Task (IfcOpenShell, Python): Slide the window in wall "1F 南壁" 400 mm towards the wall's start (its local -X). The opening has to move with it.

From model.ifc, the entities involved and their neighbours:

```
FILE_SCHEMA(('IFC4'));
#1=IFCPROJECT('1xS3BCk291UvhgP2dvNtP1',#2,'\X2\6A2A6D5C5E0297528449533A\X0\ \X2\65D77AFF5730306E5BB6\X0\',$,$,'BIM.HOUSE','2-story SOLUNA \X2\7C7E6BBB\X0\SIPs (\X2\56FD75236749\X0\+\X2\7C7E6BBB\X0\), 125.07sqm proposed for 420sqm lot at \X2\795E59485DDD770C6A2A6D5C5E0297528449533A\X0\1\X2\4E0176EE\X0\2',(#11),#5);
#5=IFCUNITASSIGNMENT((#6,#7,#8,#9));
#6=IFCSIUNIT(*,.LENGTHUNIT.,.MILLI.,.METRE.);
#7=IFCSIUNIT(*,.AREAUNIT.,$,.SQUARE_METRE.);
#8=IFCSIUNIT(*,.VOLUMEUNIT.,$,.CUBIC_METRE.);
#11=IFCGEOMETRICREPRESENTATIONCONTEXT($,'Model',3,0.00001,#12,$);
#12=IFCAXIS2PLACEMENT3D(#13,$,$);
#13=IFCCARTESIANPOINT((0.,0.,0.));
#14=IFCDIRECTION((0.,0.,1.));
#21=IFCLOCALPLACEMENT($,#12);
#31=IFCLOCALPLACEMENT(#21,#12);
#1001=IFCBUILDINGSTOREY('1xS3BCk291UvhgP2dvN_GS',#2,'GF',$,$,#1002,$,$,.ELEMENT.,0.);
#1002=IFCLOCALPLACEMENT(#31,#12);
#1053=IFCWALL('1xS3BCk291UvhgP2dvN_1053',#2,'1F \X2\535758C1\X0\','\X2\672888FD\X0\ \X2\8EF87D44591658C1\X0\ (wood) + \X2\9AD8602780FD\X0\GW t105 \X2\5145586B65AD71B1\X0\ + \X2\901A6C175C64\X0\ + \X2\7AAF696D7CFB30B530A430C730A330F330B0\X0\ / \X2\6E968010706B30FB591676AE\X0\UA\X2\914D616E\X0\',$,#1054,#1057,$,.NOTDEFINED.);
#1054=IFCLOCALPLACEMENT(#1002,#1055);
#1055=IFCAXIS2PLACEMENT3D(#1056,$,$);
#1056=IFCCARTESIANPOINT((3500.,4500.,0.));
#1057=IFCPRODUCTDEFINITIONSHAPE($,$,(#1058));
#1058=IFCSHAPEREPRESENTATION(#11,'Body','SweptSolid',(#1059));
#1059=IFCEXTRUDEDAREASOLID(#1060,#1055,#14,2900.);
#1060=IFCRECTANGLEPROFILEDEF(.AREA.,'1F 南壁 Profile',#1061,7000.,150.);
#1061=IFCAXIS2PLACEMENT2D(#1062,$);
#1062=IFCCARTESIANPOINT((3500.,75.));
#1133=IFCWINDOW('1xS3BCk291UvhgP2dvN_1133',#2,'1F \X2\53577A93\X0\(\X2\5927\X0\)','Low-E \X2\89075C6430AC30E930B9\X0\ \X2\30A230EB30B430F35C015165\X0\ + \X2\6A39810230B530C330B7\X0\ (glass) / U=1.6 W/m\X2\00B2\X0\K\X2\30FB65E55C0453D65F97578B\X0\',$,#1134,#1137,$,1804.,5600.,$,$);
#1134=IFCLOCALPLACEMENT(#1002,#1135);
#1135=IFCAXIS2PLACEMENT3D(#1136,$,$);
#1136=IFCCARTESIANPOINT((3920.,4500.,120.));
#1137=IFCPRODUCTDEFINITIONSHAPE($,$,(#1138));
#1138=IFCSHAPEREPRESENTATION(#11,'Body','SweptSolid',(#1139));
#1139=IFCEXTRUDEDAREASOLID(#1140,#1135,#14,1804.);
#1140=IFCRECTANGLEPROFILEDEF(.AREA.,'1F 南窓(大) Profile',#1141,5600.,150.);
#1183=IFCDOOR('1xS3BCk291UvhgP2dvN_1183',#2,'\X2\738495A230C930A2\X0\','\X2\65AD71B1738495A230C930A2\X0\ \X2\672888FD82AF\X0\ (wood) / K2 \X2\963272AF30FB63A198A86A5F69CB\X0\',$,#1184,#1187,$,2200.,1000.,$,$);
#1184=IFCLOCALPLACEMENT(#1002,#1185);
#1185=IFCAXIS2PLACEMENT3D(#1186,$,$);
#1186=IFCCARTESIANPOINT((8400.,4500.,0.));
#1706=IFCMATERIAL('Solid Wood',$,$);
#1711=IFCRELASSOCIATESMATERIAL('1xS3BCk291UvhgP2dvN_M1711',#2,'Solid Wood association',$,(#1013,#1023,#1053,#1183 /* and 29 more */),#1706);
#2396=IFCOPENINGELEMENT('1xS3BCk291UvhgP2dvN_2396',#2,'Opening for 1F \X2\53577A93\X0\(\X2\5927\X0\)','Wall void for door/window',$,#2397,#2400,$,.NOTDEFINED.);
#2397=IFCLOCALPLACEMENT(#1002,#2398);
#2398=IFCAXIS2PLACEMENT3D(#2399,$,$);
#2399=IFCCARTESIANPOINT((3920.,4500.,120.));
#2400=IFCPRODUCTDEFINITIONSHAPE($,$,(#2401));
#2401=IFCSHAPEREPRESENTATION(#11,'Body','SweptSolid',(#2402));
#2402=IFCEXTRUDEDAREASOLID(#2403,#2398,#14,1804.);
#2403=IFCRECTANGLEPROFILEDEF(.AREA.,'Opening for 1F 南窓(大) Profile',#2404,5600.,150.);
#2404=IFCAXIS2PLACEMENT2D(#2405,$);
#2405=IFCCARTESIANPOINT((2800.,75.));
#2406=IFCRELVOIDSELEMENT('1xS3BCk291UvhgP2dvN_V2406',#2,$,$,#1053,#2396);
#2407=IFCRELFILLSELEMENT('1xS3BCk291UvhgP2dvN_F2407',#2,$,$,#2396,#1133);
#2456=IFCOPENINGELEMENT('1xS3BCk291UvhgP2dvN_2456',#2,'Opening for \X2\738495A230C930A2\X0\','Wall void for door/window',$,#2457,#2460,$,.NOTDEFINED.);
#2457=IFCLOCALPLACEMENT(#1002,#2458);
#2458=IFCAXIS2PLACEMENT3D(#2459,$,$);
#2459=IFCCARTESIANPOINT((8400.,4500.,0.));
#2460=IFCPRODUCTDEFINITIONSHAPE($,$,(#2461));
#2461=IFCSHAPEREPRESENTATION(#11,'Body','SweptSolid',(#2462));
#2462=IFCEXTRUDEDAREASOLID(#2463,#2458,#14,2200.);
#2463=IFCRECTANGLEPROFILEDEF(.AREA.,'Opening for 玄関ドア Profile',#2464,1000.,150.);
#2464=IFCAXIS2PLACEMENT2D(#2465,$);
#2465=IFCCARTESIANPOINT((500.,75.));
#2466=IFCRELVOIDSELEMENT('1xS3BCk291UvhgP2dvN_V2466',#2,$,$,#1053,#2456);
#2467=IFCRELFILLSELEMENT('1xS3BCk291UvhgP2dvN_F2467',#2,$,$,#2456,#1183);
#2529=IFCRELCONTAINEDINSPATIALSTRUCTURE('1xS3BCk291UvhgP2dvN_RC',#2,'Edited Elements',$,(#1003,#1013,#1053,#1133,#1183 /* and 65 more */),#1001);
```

```python
import ifcopenshell
import ifcopenshell.api.geometry
import ifcopenshell.util.placement
import ifcopenshell.util.unit

model = ifcopenshell.open("model.ifc")
unit_scale = ifcopenshell.util.unit.calculate_unit_scale(model)

window = model.by_guid("1xS3BCk291UvhgP2dvN_1133")
opening = window.FillsVoids[0].RelatingOpeningElement
wall = opening.VoidsElements[0].RelatingBuildingElement

wall_matrix = ifcopenshell.util.placement.get_local_placement(wall.ObjectPlacement)
shift = wall_matrix[:3, 0] * -0.4 / unit_scale
before = ifcopenshell.util.placement.get_local_placement(window.ObjectPlacement)[:3, 3].copy()

# The window is not placed relative to its opening, so move both.
for product in (opening, window):
    matrix = ifcopenshell.util.placement.get_local_placement(product.ObjectPlacement)
    matrix[:3, 3] += shift
    ifcopenshell.api.geometry.edit_object_placement(model, product=product, matrix=matrix, is_si=False)

after = ifcopenshell.util.placement.get_local_placement(window.ObjectPlacement)[:3, 3]
print("window moved by", (after - before).round(3) + 0.0)

model.write("model_v2.ifc")
```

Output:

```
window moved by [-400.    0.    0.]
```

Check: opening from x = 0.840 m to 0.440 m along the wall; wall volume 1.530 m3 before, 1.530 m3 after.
